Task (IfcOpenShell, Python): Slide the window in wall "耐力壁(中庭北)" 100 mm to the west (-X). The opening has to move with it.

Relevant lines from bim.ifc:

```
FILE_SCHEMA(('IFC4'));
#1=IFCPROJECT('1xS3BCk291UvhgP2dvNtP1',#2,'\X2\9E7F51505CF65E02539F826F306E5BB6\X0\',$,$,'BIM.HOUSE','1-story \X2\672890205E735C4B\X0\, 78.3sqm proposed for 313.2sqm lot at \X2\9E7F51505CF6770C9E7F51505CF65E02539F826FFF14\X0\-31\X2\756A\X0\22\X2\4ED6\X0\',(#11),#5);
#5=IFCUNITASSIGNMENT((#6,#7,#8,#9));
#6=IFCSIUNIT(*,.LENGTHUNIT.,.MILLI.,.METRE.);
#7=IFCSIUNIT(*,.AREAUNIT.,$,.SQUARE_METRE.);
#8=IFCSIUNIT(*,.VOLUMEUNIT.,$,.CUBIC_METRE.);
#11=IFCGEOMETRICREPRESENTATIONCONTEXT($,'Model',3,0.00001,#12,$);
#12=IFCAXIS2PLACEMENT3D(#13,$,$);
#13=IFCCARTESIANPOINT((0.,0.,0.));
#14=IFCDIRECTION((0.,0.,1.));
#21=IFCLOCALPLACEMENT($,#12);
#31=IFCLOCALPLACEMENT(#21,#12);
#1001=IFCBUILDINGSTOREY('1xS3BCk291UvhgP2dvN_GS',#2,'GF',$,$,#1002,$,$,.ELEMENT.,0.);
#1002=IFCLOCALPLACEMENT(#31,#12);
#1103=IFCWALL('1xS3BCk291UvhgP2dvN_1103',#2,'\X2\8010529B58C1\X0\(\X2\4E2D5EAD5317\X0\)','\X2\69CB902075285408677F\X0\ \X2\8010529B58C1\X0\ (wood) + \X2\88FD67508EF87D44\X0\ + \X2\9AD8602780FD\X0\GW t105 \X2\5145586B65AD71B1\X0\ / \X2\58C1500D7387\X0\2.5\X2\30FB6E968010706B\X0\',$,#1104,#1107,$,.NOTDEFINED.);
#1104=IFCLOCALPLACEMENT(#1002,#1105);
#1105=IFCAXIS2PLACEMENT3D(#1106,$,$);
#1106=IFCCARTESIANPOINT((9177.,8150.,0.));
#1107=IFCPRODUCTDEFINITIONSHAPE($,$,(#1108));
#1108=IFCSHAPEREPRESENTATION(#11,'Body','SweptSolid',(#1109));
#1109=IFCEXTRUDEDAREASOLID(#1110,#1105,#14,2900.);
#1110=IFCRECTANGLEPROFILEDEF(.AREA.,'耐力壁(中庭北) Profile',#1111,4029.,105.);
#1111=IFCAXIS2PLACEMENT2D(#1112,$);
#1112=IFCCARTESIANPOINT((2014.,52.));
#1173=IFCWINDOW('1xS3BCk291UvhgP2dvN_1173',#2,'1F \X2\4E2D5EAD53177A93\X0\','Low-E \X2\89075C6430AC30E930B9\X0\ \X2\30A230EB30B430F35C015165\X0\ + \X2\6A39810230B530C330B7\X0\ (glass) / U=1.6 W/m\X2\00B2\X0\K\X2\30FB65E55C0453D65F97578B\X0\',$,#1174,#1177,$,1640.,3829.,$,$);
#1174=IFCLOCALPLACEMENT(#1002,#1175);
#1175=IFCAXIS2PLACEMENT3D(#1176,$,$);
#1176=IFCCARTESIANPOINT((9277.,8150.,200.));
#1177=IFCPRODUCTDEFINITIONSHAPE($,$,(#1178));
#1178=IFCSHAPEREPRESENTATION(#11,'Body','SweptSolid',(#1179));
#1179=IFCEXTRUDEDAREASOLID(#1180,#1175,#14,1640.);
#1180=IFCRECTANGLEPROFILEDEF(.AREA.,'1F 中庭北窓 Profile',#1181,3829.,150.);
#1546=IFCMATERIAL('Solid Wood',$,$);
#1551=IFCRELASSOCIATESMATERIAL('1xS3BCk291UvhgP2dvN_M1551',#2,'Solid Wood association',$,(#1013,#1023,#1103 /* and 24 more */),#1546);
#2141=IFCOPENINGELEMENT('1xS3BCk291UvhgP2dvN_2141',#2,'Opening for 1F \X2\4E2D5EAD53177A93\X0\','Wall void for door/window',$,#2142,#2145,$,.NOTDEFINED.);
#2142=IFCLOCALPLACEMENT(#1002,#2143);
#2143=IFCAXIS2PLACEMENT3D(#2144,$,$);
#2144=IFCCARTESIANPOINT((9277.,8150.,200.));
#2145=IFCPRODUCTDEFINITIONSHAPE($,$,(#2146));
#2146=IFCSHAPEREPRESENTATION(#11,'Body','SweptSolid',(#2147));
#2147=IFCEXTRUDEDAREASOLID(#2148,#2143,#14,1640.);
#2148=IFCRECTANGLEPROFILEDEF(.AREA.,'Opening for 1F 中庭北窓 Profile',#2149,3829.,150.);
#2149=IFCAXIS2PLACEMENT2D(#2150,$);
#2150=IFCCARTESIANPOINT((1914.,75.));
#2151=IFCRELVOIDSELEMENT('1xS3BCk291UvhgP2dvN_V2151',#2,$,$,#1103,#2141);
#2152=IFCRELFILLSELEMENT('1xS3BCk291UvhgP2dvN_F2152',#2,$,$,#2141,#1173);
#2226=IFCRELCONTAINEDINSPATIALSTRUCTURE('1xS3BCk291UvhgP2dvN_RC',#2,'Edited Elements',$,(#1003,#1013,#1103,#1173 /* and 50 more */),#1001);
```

```python
import ifcopenshell
import ifcopenshell.api.geometry
import ifcopenshell.util.placement
import ifcopenshell.util.unit

model = ifcopenshell.open("bim.ifc")
unit_scale = ifcopenshell.util.unit.calculate_unit_scale(model)

window = model.by_id(1173)
opening = window.FillsVoids[0].RelatingOpeningElement
wall = opening.VoidsElements[0].RelatingBuildingElement

wall_matrix = ifcopenshell.util.placement.get_local_placement(wall.ObjectPlacement)
shift = wall_matrix[:3, 0] * -0.1 / unit_scale
before = ifcopenshell.util.placement.get_local_placement(window.ObjectPlacement)[:3, 3].copy()

# The window is not placed relative to its opening, so move both.
for product in (opening, window):
    matrix = ifcopenshell.util.placement.get_local_placement(product.ObjectPlacement)
    matrix[:3, 3] += shift
    ifcopenshell.api.geometry.edit_object_placement(model, product=product, matrix=matrix, is_si=False)

after = ifcopenshell.util.placement.get_local_placement(window.ObjectPlacement)[:3, 3]
print("window moved by", (after - before).round(3) + 0.0)

model.write("bim_updated.ifc")
```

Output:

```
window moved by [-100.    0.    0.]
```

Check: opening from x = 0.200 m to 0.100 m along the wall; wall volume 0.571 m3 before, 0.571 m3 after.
